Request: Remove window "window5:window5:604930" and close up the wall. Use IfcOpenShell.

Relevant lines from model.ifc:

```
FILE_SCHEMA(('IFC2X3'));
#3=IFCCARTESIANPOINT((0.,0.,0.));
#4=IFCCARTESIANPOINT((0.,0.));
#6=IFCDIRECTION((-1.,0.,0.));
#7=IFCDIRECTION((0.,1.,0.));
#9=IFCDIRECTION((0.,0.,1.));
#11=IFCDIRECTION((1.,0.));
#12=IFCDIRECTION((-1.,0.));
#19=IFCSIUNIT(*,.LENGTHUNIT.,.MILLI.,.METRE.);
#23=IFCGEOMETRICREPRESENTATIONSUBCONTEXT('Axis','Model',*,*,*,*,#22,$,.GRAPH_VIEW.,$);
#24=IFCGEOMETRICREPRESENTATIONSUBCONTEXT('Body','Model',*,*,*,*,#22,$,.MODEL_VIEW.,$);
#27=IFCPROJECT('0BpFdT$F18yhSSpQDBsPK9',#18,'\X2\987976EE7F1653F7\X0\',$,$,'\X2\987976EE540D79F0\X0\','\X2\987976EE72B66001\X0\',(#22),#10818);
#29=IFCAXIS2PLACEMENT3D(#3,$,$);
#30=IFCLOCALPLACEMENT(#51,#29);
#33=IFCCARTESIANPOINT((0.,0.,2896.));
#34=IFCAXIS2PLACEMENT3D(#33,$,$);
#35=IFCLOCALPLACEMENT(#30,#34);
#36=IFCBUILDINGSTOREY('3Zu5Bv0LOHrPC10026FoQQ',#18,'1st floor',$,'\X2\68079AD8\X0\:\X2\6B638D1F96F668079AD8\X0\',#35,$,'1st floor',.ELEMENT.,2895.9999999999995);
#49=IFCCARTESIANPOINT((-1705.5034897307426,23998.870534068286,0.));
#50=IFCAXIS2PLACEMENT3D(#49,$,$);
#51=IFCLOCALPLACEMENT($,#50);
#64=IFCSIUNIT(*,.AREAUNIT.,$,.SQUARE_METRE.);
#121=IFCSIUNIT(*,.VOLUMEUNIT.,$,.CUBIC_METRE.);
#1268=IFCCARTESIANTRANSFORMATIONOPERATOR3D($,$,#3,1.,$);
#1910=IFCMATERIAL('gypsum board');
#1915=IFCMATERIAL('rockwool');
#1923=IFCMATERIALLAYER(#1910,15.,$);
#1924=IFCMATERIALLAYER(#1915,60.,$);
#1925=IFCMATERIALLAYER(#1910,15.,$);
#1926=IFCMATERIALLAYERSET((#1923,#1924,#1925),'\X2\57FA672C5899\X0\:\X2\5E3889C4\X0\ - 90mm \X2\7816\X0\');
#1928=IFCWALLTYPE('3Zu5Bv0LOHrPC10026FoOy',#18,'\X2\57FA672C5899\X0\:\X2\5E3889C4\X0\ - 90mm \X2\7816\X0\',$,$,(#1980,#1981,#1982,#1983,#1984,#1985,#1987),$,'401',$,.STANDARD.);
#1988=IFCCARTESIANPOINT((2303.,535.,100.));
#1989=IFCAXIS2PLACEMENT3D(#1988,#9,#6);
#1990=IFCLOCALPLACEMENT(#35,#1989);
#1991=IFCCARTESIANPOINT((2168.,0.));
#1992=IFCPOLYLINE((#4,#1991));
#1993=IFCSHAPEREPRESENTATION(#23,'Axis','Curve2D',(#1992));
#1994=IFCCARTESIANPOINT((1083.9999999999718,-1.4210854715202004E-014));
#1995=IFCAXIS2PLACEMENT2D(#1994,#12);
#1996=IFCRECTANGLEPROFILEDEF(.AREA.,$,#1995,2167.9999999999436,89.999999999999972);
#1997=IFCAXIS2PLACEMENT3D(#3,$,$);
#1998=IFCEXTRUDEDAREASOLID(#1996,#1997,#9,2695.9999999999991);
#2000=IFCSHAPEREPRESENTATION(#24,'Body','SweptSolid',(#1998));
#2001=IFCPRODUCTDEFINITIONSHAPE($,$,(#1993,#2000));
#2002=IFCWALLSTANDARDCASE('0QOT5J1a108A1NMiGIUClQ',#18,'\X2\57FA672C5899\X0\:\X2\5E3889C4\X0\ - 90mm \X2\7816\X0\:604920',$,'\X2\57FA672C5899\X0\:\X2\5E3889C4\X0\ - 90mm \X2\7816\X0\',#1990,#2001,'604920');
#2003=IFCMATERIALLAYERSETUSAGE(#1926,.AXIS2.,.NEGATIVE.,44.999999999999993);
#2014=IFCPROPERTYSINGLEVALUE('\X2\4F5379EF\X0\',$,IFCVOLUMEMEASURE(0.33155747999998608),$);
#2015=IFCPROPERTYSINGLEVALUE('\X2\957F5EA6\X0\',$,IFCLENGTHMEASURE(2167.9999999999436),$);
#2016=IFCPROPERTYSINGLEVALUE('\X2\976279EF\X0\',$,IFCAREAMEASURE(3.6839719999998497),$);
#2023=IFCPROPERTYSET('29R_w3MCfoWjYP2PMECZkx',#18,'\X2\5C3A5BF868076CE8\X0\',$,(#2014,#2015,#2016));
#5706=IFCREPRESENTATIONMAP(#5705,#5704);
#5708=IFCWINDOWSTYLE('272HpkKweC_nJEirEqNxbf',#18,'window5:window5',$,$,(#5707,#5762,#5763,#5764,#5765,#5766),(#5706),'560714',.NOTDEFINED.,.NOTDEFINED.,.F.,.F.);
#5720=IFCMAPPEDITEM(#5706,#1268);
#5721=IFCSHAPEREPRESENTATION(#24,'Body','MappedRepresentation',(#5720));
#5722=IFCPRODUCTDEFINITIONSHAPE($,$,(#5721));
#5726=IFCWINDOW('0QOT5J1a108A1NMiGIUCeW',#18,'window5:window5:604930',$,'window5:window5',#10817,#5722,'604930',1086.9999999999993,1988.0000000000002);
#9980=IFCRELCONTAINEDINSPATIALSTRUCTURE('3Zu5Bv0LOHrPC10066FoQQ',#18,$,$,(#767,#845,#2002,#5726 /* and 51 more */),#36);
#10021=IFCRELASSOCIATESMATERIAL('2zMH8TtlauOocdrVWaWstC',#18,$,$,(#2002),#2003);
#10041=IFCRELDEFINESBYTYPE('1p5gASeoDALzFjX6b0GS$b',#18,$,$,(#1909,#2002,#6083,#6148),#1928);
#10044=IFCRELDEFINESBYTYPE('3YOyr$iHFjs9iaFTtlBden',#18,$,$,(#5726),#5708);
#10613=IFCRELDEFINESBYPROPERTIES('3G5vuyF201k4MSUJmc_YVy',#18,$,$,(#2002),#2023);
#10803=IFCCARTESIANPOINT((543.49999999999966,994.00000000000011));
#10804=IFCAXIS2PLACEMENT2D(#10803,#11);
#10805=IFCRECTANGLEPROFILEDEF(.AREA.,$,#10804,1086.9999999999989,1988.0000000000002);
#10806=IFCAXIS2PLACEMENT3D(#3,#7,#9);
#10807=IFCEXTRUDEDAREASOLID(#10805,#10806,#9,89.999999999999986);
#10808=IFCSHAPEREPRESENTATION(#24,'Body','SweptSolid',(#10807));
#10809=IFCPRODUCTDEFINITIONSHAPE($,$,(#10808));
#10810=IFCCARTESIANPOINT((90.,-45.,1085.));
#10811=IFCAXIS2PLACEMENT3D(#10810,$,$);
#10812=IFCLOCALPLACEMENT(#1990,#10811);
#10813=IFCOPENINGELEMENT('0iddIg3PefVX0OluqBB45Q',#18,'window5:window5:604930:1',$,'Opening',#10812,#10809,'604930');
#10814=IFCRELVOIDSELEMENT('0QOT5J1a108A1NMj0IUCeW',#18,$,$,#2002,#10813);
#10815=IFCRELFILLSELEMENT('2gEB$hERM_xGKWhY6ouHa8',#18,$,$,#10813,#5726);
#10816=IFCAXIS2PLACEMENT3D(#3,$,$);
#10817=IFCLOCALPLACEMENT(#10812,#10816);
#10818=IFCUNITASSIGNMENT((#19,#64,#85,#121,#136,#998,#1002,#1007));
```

```python
import ifcopenshell
import ifcopenshell.api.feature
import ifcopenshell.api.pset
import ifcopenshell.api.root
import ifcopenshell.geom
import ifcopenshell.util.element
import ifcopenshell.util.shape
import ifcopenshell.util.unit

model = ifcopenshell.open("model.ifc")
area_scale = ifcopenshell.util.unit.calculate_unit_scale(model, "AREAUNIT")
volume_scale = ifcopenshell.util.unit.calculate_unit_scale(model, "VOLUMEUNIT")
settings = ifcopenshell.geom.settings()


def volume(element):
    """Net volume in cubic metres, openings subtracted."""
    shape = ifcopenshell.geom.create_shape(settings, element)
    return ifcopenshell.util.shape.get_volume(shape.geometry)


window = model.by_guid("0QOT5J1a108A1NMiGIUCeW")
opening = window.FillsVoids[0].RelatingOpeningElement
wall = opening.VoidsElements[0].RelatingBuildingElement
before = volume(wall)

ifcopenshell.api.root.remove_product(model, product=window)
ifcopenshell.api.feature.remove_feature(model, feature=opening)

after = volume(wall)
thickness = 0.09  # wall thickness in metres

# Update the wall's stored quantities.
pset = model.by_id(ifcopenshell.util.element.get_pset(wall, "尺寸标注", should_inherit=False)["id"])
ifcopenshell.api.pset.edit_pset(model, pset=pset, properties={
    "体积": model.create_entity("IfcVolumeMeasure", after / volume_scale),
    "面积": model.create_entity("IfcAreaMeasure", after / thickness / area_scale),
})

print(f"wall volume {before:.3f} -> {after:.3f} m3")

model.write("model-out.ifc")
```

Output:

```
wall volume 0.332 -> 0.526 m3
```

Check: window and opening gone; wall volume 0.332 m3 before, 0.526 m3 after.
